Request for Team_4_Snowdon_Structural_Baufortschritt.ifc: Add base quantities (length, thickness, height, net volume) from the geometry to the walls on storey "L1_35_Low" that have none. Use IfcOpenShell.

First a look at what the model holds.

```python
import ifcopenshell
import ifcopenshell.util.element
import ifcopenshell.util.unit

model = ifcopenshell.open("Team_4_Snowdon_Structural_Baufortschritt.ifc")
print(model.schema)
for unit_type in ("LENGTHUNIT", "AREAUNIT", "VOLUMEUNIT"):
    print(unit_type, ifcopenshell.util.unit.calculate_unit_scale(model, unit_type))
storey = next(s for s in model.by_type("IfcBuildingStorey") if s.Name == "L1_35_Low")
walls = [e for e in ifcopenshell.util.element.get_decomposition(storey) if e.is_a("IfcWall")]
for e in sorted(walls, key=lambda e: e.id()):
    print(e.id(), e.is_a(), e.Name, list(ifcopenshell.util.element.get_psets(e, qtos_only=True)), sep=" | ")
```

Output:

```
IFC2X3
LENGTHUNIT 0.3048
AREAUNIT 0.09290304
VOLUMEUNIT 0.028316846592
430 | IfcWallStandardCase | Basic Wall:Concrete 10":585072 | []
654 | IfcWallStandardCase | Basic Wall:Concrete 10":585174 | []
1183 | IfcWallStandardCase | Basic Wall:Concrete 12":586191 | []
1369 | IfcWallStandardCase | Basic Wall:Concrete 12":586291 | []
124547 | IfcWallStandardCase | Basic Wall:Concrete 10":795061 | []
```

```python
import ifcopenshell
import ifcopenshell.api.pset
import ifcopenshell.geom
import ifcopenshell.util.element
import ifcopenshell.util.shape
import ifcopenshell.util.unit

model = ifcopenshell.open("Team_4_Snowdon_Structural_Baufortschritt.ifc")
unit_scale = ifcopenshell.util.unit.calculate_unit_scale(model)
volume_scale = ifcopenshell.util.unit.calculate_unit_scale(model, "VOLUMEUNIT")
settings = ifcopenshell.geom.settings()

storey = next(s for s in model.by_type("IfcBuildingStorey") if s.Name == "L1_35_Low")
walls = [e for e in ifcopenshell.util.element.get_decomposition(storey) if e.is_a("IfcWall")]

for e in sorted(walls, key=lambda e: e.id()):
    if ifcopenshell.util.element.get_psets(e, qtos_only=True, should_inherit=False):
        continue
    # Geometry comes back in metres, in the element's own axes.
    shape = ifcopenshell.geom.create_shape(settings, e)
    values = {
        "Length": ifcopenshell.util.shape.get_x(shape.geometry) / unit_scale,
        "Width": ifcopenshell.util.shape.get_y(shape.geometry) / unit_scale,
        "Height": ifcopenshell.util.shape.get_z(shape.geometry) / unit_scale,
        "NetVolume": ifcopenshell.util.shape.get_volume(shape.geometry) / volume_scale,
    }
    qto = ifcopenshell.api.pset.add_qto(model, product=e, name="BaseQuantities")
    ifcopenshell.api.pset.edit_qto(model, qto=qto, properties=values)
    print(e.id(), {k: round(v, 3) for k, v in values.items()})

model.write("Team_4_Snowdon_Structural_Baufortschritt_v2.ifc")
```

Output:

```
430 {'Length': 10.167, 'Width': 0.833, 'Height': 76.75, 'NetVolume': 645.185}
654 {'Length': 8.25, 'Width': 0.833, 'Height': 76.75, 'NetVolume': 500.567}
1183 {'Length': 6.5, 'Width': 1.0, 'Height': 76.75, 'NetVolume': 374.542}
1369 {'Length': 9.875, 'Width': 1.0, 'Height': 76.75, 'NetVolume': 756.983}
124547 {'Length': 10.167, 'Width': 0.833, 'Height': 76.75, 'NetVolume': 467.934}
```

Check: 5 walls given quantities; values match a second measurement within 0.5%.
